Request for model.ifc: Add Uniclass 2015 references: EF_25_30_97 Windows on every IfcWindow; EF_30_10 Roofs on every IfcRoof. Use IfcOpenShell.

First a look at what the model holds.

```python
import ifcopenshell

model = ifcopenshell.open("model.ifc")
print(model.schema)
print("classifications:", [c.Name for c in model.by_type("IfcClassification")])
for ifc_class in ("IfcDoor", "IfcRoof", "IfcStair", "IfcWall", "IfcWindow"):
    print(ifc_class, len(model.by_type(ifc_class)))
```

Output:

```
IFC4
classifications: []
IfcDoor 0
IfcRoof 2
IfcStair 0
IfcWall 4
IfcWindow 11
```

```python
import ifcopenshell
import ifcopenshell.api.classification

model = ifcopenshell.open("model.ifc")

system = ifcopenshell.api.classification.add_classification(model, classification="Uniclass 2015")

codes = {
    "IfcWindow": ("EF_25_30_97", "Windows"),
    "IfcRoof": ("EF_30_10", "Roofs"),
}
for ifc_class, (code, name) in codes.items():
    products = model.by_type(ifc_class)
    ifcopenshell.api.classification.add_reference(
        model, products=products, classification=system, identification=code, name=name
    )
    print(code, len(products))

model.write("model_v2.ifc")
```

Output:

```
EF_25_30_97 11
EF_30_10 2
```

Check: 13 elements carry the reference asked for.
